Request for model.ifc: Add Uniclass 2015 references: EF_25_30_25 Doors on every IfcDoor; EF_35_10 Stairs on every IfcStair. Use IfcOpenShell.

First a look at what the model holds.

```python
import ifcopenshell

model = ifcopenshell.open("model.ifc")
print(model.schema)
print("classifications:", [c.Name for c in model.by_type("IfcClassification")])
for ifc_class in ("IfcDoor", "IfcRoof", "IfcStair", "IfcWall", "IfcWindow"):
    print(ifc_class, len(model.by_type(ifc_class)))
```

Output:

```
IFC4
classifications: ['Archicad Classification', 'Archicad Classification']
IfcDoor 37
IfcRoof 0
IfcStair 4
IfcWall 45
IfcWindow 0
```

```python
import ifcopenshell
import ifcopenshell.api.classification

model = ifcopenshell.open("model.ifc")

system = ifcopenshell.api.classification.add_classification(model, classification="Uniclass 2015")

codes = {
    "IfcDoor": ("EF_25_30_25", "Doors"),
    "IfcStair": ("EF_35_10", "Stairs"),
}
for ifc_class, (code, name) in codes.items():
    products = model.by_type(ifc_class)
    ifcopenshell.api.classification.add_reference(
        model, products=products, classification=system, identification=code, name=name
    )
    print(code, len(products))

model.write("model-out.ifc")
```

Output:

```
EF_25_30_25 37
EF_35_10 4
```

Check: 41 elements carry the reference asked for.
